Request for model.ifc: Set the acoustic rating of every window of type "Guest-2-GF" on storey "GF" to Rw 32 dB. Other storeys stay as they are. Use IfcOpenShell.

First a look at what the model holds.

```python
import ifcopenshell
import ifcopenshell.util.element

model = ifcopenshell.open("model.ifc")
print(model.schema)
storey = next(s for s in model.by_type("IfcBuildingStorey") if s.Name == "GF")
windows = [e for e in ifcopenshell.util.element.get_decomposition(storey) if e.is_a("IfcWindow")]
seen = {}
for e in windows:
    element_type = ifcopenshell.util.element.get_type(e)
    key = (element_type.Name if element_type != e and element_type else None, ifcopenshell.util.element.get_pset(e, "Pset_WindowCommon", "AcousticRating"))
    seen[key] = seen.get(key, 0) + 1
for (name, value), count in sorted(seen.items(), key=str):
    print(count, "x", name, "|", value)
```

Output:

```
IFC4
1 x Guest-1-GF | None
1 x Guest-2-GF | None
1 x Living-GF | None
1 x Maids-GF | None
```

```python
import ifcopenshell
import ifcopenshell.api.pset
import ifcopenshell.util.element

model = ifcopenshell.open("model.ifc")

storey = next(s for s in model.by_type("IfcBuildingStorey") if s.Name == "GF")
windows = [e for e in ifcopenshell.util.element.get_decomposition(storey) if e.is_a("IfcWindow")]

count = 0
for e in windows:
    element_type = ifcopenshell.util.element.get_type(e)
    if element_type in (None, e) or element_type.Name != "Guest-2-GF":
        continue
    # add_pset returns the element's existing set when there is one.
    pset = ifcopenshell.api.pset.add_pset(model, product=e, name="Pset_WindowCommon")
    ifcopenshell.api.pset.edit_pset(model, pset=pset, properties={"AcousticRating": "Rw 32 dB"})
    count += 1

print(count, "windows updated")

model.write("model-out.ifc")
```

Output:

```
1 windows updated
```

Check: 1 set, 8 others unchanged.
